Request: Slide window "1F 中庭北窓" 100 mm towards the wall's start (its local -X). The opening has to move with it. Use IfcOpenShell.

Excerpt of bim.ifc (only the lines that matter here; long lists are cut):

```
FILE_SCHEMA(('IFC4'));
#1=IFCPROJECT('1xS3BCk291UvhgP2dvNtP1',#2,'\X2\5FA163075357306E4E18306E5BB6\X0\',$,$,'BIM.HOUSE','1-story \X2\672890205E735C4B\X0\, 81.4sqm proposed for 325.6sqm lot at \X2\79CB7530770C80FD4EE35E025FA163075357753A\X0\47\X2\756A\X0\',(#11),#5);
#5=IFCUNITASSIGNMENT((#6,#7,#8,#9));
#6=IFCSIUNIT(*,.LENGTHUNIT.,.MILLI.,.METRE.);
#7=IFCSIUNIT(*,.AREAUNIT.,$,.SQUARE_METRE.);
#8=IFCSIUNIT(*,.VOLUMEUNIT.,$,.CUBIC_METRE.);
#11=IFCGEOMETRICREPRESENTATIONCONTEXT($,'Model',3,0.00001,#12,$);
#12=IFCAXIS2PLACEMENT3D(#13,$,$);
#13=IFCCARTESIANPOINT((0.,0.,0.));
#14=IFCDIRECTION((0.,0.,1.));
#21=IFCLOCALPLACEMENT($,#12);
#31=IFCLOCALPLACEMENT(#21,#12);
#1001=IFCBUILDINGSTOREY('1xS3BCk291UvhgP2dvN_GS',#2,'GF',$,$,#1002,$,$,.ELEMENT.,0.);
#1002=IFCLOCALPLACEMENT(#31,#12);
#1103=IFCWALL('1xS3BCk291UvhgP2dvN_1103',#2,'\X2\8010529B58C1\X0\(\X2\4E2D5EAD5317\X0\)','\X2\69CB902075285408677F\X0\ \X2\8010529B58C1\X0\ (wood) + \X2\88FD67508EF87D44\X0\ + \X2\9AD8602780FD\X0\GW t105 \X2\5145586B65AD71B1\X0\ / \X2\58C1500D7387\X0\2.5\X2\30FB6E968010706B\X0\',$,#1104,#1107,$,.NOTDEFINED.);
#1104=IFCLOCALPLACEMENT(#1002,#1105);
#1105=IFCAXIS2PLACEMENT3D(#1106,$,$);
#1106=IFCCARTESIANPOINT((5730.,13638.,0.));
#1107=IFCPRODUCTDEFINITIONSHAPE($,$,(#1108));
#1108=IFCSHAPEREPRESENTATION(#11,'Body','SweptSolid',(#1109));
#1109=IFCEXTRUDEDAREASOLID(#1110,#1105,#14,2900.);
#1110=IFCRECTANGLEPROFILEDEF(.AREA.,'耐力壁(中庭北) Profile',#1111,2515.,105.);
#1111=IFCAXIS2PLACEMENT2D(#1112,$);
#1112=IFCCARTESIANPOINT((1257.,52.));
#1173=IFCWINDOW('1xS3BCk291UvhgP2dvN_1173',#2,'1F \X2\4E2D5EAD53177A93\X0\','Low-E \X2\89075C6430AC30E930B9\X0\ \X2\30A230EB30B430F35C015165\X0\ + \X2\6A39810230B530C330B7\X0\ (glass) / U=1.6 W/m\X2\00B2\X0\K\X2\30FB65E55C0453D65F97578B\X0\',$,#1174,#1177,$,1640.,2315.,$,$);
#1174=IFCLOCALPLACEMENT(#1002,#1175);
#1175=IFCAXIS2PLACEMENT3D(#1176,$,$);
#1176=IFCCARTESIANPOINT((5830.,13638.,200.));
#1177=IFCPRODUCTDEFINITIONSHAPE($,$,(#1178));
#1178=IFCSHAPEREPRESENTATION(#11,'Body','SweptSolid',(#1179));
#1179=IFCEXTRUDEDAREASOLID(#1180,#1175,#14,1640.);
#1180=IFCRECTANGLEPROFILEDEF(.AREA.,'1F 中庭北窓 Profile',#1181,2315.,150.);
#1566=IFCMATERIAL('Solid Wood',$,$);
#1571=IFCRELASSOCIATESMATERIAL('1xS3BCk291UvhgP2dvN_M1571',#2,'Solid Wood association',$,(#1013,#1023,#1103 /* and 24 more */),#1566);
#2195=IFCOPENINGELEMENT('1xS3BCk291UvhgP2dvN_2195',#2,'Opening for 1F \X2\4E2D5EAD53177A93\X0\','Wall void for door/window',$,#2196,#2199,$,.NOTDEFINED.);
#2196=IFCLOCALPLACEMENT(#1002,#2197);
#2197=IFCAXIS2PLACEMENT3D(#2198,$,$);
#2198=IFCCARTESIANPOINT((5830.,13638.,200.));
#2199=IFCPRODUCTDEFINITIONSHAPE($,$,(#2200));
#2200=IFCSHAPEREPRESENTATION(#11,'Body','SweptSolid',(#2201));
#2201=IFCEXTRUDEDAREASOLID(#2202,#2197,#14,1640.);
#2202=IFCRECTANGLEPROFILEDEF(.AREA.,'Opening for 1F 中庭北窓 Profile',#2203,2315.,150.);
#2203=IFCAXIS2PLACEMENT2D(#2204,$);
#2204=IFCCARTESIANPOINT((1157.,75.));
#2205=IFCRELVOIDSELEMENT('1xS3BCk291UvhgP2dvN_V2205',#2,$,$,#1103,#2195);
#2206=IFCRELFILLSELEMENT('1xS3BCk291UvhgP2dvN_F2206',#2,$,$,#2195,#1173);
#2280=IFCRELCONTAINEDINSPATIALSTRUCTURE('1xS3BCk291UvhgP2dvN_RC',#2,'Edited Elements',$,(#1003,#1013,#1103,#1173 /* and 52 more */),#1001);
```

```python
import ifcopenshell
import ifcopenshell.api.geometry
import ifcopenshell.util.placement
import ifcopenshell.util.unit

model = ifcopenshell.open("bim.ifc")
unit_scale = ifcopenshell.util.unit.calculate_unit_scale(model)

window = model.by_id(1173)
opening = window.FillsVoids[0].RelatingOpeningElement
wall = opening.VoidsElements[0].RelatingBuildingElement

wall_matrix = ifcopenshell.util.placement.get_local_placement(wall.ObjectPlacement)
shift = wall_matrix[:3, 0] * -0.1 / unit_scale
before = ifcopenshell.util.placement.get_local_placement(window.ObjectPlacement)[:3, 3].copy()

# The window is not placed relative to its opening, so move both.
for product in (opening, window):
    matrix = ifcopenshell.util.placement.get_local_placement(product.ObjectPlacement)
    matrix[:3, 3] += shift
    ifcopenshell.api.geometry.edit_object_placement(model, product=product, matrix=matrix, is_si=False)

after = ifcopenshell.util.placement.get_local_placement(window.ObjectPlacement)[:3, 3]
print("window moved by", (after - before).round(3) + 0.0)

model.write("bim-out.ifc")
```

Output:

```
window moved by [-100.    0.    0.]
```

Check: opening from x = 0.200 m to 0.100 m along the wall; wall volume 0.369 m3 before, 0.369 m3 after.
